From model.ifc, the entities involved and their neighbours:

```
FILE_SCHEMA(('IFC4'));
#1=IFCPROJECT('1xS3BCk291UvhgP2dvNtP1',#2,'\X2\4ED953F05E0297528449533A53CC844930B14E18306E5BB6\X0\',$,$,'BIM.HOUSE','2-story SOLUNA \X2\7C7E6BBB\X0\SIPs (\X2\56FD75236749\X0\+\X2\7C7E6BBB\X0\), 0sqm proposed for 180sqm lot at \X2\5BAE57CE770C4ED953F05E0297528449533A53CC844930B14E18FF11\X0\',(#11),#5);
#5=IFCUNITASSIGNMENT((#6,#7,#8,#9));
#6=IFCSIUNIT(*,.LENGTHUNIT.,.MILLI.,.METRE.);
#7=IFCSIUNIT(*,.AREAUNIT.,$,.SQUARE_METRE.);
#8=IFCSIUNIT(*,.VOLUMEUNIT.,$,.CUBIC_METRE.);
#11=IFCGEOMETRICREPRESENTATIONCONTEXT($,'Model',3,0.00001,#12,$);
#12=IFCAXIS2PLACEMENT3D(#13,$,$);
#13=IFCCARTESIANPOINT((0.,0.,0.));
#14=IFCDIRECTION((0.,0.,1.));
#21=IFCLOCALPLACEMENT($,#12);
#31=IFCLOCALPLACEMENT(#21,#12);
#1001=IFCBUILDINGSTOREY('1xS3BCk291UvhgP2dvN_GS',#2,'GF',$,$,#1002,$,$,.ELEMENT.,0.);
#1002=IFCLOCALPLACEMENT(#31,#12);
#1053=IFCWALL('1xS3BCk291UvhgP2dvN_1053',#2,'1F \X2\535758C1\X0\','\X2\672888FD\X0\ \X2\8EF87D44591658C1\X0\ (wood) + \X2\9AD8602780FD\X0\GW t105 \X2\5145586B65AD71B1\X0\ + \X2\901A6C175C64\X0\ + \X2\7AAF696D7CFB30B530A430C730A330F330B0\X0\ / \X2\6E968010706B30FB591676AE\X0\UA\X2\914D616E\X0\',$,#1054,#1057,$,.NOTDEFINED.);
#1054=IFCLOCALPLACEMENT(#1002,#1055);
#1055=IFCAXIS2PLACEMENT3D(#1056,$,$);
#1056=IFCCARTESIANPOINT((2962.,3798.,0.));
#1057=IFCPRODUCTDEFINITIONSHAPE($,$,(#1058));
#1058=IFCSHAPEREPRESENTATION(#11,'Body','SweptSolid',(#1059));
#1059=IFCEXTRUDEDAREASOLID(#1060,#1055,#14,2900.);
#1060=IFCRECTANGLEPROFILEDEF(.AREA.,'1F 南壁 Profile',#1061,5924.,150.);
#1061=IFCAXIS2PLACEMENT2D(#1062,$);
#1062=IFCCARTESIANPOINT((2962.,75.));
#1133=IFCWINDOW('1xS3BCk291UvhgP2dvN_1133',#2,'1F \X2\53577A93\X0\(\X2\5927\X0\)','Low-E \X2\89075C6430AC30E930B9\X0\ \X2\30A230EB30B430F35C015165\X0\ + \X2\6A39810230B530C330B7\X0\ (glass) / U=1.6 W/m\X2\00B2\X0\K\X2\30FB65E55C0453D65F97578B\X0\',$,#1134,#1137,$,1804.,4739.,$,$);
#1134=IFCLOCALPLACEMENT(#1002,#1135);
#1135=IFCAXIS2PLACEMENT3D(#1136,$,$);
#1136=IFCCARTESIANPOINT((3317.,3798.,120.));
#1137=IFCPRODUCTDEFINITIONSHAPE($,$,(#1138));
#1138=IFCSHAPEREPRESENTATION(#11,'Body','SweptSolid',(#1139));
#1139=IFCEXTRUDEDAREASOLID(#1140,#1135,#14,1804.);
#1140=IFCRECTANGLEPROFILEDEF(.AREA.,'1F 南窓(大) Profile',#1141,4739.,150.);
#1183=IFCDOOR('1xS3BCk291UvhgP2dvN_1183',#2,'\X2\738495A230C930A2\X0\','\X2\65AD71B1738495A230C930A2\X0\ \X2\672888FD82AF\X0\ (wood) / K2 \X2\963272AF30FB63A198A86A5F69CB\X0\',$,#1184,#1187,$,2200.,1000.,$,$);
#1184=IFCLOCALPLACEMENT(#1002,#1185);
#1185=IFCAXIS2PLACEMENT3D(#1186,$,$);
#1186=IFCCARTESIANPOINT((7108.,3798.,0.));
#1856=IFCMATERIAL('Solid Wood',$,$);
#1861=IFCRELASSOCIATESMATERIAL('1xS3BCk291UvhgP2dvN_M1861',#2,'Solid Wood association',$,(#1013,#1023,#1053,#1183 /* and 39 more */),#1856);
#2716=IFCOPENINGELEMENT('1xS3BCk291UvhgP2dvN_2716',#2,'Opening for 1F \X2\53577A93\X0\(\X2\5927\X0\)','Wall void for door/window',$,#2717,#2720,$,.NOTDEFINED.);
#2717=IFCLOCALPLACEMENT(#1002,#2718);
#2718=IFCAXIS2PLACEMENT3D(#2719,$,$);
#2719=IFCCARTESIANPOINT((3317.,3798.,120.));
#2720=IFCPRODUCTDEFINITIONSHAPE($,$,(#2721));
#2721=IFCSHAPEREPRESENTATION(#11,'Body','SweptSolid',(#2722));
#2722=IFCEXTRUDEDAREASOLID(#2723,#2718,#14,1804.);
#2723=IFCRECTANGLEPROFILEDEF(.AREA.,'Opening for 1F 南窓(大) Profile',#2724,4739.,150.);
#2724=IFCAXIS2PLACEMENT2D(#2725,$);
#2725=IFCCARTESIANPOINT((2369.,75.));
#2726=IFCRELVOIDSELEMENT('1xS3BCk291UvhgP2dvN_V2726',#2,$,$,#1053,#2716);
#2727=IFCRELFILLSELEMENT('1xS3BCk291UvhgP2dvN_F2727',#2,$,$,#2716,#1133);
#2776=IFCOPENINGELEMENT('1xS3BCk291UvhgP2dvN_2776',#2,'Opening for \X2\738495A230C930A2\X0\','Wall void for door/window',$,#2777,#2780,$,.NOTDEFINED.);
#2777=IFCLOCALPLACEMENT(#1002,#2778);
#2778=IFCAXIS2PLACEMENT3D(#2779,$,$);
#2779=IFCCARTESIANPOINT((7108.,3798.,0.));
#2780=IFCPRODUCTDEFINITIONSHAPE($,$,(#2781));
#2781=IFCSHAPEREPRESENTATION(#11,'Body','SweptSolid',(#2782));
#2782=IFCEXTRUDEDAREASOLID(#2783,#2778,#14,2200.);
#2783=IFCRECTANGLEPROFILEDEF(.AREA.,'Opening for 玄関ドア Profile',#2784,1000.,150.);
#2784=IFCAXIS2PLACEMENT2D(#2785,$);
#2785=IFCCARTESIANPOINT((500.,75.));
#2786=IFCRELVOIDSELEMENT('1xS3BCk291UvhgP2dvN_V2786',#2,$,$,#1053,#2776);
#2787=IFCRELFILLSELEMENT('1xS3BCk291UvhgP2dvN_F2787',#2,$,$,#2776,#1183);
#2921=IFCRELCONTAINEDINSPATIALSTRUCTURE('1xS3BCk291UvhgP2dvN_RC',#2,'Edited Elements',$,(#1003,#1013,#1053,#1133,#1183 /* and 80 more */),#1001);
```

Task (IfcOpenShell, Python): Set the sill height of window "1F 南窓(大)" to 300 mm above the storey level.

```python
import numpy as np
import ifcopenshell
import ifcopenshell.api.geometry
import ifcopenshell.geom
import ifcopenshell.util.element
import ifcopenshell.util.placement
import ifcopenshell.util.shape
import ifcopenshell.util.unit

model = ifcopenshell.open("model.ifc")
unit_scale = ifcopenshell.util.unit.calculate_unit_scale(model)

window = model.by_guid("1xS3BCk291UvhgP2dvN_1133")
opening = window.FillsVoids[0].RelatingOpeningElement
storey = ifcopenshell.util.element.get_container(window, ifc_class="IfcBuildingStorey")
level = ifcopenshell.util.placement.get_local_placement(storey.ObjectPlacement)[2, 3]

# The opening's origin need not be at the sill, so measure its lowest point.
shape = ifcopenshell.geom.create_shape(ifcopenshell.geom.settings(), opening)
bottom = ifcopenshell.util.shape.get_shape_bottom_elevation(shape, shape.geometry) / unit_scale
dz = level + 300.0 - bottom

shift = np.array([0.0, 0.0, dz])
# The window is not placed relative to its opening, so move both.
for product in (opening, window):
    matrix = ifcopenshell.util.placement.get_local_placement(product.ObjectPlacement)
    matrix[:3, 3] += shift
    ifcopenshell.api.geometry.edit_object_placement(model, product=product, matrix=matrix, is_si=False)

print(f"moved by {dz * unit_scale:+.3f} m")

model.write("model_rev.ifc")
```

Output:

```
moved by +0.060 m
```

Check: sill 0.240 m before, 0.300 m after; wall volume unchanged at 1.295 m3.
